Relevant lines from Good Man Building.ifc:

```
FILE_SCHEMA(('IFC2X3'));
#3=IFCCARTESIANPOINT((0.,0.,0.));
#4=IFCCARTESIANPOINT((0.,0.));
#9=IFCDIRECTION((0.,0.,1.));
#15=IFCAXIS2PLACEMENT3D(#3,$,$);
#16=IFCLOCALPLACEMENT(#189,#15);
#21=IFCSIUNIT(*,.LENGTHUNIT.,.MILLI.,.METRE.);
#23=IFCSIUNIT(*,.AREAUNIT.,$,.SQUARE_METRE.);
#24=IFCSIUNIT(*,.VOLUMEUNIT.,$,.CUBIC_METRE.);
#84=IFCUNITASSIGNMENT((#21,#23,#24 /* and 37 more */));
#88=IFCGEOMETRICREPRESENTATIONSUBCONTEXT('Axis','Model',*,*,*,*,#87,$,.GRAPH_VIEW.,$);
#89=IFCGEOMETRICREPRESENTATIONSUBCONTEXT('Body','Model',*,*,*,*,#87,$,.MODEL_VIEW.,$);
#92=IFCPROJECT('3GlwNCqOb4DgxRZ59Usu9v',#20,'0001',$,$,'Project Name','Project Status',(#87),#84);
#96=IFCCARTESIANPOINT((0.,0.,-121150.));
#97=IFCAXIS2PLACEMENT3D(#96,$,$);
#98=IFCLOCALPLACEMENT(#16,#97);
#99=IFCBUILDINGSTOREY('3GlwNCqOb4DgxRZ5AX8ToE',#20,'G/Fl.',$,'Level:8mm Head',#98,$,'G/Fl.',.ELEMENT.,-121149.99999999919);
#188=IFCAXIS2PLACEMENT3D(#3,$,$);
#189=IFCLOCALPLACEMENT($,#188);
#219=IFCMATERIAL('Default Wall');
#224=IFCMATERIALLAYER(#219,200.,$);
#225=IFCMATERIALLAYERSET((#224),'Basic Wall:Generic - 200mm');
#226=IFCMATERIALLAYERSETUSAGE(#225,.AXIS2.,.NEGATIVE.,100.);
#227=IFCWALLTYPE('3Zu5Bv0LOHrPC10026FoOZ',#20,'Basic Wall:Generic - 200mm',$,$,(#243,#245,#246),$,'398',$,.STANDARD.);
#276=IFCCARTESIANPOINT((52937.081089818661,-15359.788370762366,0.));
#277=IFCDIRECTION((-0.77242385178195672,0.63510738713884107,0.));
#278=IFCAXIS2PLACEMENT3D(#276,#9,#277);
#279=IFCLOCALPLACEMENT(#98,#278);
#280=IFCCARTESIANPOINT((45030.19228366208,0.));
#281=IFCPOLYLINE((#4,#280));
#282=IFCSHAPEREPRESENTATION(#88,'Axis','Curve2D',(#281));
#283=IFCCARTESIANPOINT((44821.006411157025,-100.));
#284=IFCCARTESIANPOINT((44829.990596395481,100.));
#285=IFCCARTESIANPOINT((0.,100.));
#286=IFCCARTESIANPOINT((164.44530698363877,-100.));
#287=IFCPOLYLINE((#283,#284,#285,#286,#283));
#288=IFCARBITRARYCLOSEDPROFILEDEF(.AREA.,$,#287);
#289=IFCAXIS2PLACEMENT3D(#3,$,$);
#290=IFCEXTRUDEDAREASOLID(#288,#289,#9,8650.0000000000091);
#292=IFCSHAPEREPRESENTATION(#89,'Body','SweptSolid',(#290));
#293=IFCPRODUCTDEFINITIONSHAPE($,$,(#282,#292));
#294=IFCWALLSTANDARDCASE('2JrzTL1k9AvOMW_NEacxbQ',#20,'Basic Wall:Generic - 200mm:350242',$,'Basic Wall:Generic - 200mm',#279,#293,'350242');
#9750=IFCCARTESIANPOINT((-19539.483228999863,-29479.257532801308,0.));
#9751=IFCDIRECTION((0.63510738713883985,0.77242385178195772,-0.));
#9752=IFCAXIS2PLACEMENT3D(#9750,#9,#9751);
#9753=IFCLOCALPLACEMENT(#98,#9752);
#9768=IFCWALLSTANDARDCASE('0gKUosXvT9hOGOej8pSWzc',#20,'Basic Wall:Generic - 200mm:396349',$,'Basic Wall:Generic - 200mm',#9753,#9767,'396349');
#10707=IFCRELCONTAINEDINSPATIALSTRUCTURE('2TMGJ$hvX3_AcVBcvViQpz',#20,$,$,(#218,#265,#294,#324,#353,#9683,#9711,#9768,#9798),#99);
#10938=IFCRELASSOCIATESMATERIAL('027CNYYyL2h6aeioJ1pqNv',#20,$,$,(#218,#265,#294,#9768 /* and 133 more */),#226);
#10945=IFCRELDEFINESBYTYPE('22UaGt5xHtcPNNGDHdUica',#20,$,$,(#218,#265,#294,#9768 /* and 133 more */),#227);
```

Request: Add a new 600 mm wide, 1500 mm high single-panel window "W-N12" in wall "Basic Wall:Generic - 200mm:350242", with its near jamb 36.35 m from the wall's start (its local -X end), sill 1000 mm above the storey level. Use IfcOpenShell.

```python
import numpy as np
import ifcopenshell
import ifcopenshell.api.feature
import ifcopenshell.api.geometry
import ifcopenshell.api.root
import ifcopenshell.api.spatial
import ifcopenshell.api.type
import ifcopenshell.geom
import ifcopenshell.util.element
import ifcopenshell.util.placement
import ifcopenshell.util.representation
import ifcopenshell.util.shape
import ifcopenshell.util.unit

model = ifcopenshell.open("Good Man Building.ifc")
unit_scale = ifcopenshell.util.unit.calculate_unit_scale(model)
settings = ifcopenshell.geom.settings()


def volume(element):
    """Net volume in cubic metres, openings subtracted."""
    shape = ifcopenshell.geom.create_shape(settings, element)
    return ifcopenshell.util.shape.get_volume(shape.geometry)


wall = model.by_id(294)
storey = ifcopenshell.util.element.get_container(wall, ifc_class="IfcBuildingStorey")
context = ifcopenshell.util.representation.get_context(model, "Model", "Body", "MODEL_VIEW")
before = volume(wall)

width, height, from_end, sill = 0.6, 1.5, 36.35, 1  # metres

# The wall runs along its own X axis, and the end named is its -X end.
wall_shape = ifcopenshell.geom.create_shape(settings, wall)
x, y, z = ifcopenshell.util.shape.get_vertices(wall_shape.geometry).T
start = x.min() + from_end
face, thickness = float(y.min()), float(y.max() - y.min())
wall_matrix = ifcopenshell.util.placement.get_local_placement(wall.ObjectPlacement)
level = ifcopenshell.util.placement.get_local_placement(storey.ObjectPlacement)[2, 3]


def in_wall(x, y):
    """Placement at x, y metres in the wall's axes, at sill height."""
    matrix = wall_matrix.copy()
    matrix[:, 3] = wall_matrix @ np.array([x / unit_scale, y / unit_scale, 0.0, 1.0])
    matrix[2, 3] = level + sill / unit_scale
    return matrix


# Opening: a box that overshoots both wall faces by 50 mm.
opening = ifcopenshell.api.root.create_entity(model, ifc_class="IfcOpeningElement")
box = ifcopenshell.api.geometry.add_wall_representation(
    model, context=context, length=width, height=height, thickness=thickness + 0.1
)
ifcopenshell.api.geometry.assign_representation(model, product=opening, representation=box)
ifcopenshell.api.geometry.edit_object_placement(model, product=opening, matrix=in_wall(start, face - 0.05), is_si=False)
ifcopenshell.api.feature.add_feature(model, feature=opening, element=wall)

window = ifcopenshell.api.root.create_entity(model, ifc_class="IfcWindow", name="W-N12")
window.OverallWidth, window.OverallHeight = width / unit_scale, height / unit_scale
body = ifcopenshell.api.geometry.add_window_representation(
    model,
    context=context,
    overall_width=window.OverallWidth,
    overall_height=window.OverallHeight,
    partition_type="SINGLE_PANEL",
)
ifcopenshell.api.geometry.assign_representation(model, product=window, representation=body)
ifcopenshell.api.spatial.assign_container(model, products=[window], relating_structure=storey)
fills = ifcopenshell.api.feature.add_filling(model, opening=opening, element=window)
fills.OwnerHistory = window.OwnerHistory  # required in IFC2X3

# IFC2X3 keeps the operation on the window style.
style = ifcopenshell.api.root.create_entity(model, ifc_class="IfcWindowStyle", name="W-N12")
style.OperationType, style.ConstructionType = "SINGLE_PANEL", "NOTDEFINED"
style.ParameterTakesPrecedence = style.Sizeable = False
ifcopenshell.api.type.assign_type(model, related_objects=[window], relating_type=style)

# Centre the window in the wall's thickness.
ifcopenshell.api.geometry.edit_object_placement(model, product=window, matrix=in_wall(start, face), is_si=False)
window_shape = ifcopenshell.geom.create_shape(settings, window)
depth = ifcopenshell.util.shape.get_vertices(window_shape.geometry)[:, 1]
offset = face + thickness / 2 - (depth.min() + depth.max()) / 2
ifcopenshell.api.geometry.edit_object_placement(model, product=window, matrix=in_wall(start, offset), is_si=False)

after = volume(wall)

print(f"wall volume {before:.3f} -> {after:.3f} m3")

model.write("Good Man Building_rev.ifc")
```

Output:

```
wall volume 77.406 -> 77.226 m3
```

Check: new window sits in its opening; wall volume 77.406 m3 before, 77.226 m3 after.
